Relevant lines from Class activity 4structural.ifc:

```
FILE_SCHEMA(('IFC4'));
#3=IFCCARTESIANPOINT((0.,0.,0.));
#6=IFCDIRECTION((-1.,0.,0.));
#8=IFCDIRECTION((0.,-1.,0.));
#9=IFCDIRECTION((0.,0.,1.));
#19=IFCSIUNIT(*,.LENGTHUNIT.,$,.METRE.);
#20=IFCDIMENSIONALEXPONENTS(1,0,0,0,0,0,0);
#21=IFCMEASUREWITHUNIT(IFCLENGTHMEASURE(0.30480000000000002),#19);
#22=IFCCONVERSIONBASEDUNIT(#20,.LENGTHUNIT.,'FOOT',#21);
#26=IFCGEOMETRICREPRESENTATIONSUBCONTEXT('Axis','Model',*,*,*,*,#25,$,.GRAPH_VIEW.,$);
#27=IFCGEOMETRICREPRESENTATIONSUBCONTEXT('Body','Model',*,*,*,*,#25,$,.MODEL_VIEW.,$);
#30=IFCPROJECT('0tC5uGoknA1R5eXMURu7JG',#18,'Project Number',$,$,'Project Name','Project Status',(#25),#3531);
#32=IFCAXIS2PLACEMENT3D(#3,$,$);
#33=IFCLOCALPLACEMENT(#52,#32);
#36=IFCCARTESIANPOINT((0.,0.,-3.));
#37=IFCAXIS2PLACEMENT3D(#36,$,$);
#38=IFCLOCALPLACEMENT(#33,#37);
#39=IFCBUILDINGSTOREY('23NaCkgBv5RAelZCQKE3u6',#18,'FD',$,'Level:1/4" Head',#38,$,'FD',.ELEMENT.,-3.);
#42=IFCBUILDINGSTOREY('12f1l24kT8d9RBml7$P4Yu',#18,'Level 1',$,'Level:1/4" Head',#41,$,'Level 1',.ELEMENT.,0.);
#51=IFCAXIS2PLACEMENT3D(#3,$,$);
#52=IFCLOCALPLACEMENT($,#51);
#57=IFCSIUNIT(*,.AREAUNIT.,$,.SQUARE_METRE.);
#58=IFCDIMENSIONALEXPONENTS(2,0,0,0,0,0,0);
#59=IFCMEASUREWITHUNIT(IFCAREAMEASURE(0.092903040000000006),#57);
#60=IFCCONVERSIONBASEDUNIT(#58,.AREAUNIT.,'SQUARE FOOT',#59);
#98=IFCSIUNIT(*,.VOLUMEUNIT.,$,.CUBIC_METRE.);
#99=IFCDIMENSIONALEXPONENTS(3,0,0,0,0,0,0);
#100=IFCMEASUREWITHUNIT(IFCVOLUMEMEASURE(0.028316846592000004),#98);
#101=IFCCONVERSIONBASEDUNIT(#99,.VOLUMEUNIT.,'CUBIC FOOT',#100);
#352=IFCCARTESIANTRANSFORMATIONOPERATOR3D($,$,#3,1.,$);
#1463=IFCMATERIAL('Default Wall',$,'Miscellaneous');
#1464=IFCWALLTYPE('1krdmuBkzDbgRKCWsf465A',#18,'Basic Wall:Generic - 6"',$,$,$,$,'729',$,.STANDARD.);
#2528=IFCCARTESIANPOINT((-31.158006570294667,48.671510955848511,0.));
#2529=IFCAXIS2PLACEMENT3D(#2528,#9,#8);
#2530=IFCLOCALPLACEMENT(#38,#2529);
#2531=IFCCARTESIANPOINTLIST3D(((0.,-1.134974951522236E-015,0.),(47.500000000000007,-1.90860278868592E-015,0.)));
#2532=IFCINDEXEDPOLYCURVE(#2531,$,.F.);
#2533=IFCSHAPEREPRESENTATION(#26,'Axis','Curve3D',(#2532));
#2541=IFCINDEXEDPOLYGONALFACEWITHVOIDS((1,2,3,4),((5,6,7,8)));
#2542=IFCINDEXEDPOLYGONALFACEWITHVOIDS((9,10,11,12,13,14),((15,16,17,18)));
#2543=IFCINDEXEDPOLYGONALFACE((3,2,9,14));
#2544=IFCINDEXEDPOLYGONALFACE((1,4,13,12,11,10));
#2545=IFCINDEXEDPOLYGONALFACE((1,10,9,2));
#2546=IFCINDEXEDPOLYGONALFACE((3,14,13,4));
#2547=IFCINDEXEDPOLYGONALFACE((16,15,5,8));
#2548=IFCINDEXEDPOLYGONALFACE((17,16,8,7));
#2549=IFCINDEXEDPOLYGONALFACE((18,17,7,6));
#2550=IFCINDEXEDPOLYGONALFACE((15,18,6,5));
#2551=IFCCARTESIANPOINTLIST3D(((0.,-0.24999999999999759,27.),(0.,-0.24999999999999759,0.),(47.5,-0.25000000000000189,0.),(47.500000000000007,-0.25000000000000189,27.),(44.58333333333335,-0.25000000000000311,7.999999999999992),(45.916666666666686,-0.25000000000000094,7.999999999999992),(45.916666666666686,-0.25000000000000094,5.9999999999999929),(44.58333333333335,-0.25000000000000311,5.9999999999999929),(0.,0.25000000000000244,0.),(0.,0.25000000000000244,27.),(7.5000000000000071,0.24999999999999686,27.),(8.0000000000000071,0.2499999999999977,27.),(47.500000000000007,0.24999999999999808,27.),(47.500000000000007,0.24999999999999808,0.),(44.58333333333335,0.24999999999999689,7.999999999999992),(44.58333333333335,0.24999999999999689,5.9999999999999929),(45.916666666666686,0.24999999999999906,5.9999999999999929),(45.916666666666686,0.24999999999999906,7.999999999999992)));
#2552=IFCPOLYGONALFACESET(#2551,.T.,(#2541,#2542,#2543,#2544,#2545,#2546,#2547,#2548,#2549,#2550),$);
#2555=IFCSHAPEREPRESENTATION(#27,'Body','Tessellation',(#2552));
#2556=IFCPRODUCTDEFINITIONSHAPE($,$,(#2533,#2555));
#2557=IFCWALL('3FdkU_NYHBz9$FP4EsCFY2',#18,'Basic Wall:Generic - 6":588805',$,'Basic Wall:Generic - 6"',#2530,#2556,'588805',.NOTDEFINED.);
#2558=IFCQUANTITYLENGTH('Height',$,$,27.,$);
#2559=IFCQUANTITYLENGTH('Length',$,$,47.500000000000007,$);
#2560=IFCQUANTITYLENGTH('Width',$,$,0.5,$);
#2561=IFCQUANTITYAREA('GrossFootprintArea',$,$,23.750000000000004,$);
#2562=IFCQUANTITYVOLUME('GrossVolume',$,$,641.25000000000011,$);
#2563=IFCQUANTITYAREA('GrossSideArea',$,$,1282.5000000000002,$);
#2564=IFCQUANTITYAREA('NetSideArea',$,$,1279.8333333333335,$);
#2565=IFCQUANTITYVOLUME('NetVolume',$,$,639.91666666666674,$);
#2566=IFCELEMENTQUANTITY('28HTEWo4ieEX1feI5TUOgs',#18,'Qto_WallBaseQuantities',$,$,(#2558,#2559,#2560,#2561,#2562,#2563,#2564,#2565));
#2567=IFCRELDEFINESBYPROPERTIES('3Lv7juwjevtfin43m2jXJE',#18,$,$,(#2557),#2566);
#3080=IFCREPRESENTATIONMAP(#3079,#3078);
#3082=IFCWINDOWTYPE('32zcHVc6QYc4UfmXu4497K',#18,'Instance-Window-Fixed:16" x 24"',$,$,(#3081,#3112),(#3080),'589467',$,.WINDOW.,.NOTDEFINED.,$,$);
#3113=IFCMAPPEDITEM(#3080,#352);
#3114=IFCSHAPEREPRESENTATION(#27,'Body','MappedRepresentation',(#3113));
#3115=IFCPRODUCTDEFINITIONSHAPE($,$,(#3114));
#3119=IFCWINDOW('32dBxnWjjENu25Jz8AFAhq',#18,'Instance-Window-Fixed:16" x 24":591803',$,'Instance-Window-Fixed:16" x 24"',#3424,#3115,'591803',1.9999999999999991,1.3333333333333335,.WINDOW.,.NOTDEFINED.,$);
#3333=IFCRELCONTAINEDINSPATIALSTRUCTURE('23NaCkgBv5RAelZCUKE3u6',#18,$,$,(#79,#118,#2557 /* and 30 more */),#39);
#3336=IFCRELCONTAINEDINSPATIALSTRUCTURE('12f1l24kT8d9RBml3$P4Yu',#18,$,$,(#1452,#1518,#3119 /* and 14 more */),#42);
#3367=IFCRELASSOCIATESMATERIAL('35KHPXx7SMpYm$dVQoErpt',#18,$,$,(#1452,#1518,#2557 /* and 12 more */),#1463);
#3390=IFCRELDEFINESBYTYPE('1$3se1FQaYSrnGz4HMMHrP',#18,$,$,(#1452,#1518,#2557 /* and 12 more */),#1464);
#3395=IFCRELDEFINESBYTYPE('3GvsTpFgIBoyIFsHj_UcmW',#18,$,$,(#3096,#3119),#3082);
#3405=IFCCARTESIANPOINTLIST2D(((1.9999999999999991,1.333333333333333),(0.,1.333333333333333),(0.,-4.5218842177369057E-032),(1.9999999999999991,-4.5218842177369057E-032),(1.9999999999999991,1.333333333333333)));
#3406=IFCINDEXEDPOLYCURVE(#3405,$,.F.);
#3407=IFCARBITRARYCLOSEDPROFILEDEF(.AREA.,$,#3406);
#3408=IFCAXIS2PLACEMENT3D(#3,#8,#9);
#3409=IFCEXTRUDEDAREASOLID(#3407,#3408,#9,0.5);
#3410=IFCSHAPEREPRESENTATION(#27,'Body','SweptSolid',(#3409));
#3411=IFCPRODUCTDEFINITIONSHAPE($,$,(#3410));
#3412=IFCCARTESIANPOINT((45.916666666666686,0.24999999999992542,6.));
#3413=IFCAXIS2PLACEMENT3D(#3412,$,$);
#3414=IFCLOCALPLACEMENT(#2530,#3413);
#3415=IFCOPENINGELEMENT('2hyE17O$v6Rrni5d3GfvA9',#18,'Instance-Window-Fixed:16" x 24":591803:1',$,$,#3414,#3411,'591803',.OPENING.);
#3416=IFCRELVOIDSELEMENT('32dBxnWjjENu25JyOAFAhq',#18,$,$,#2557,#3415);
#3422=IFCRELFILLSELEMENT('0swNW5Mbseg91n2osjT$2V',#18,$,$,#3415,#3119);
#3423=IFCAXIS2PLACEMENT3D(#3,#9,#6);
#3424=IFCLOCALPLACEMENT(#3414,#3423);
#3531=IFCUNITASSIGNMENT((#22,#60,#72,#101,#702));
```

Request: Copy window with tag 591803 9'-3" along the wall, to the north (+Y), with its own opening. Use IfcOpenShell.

```python
import ifcopenshell
import ifcopenshell.api.feature
import ifcopenshell.api.geometry
import ifcopenshell.api.pset
import ifcopenshell.api.root
import ifcopenshell.geom
import ifcopenshell.util.element
import ifcopenshell.util.placement
import ifcopenshell.util.shape
import ifcopenshell.util.unit

model = ifcopenshell.open("Class activity 4structural.ifc")
unit_scale = ifcopenshell.util.unit.calculate_unit_scale(model)
area_scale = ifcopenshell.util.unit.calculate_unit_scale(model, "AREAUNIT")
volume_scale = ifcopenshell.util.unit.calculate_unit_scale(model, "VOLUMEUNIT")
settings = ifcopenshell.geom.settings()


def volume(element):
    """Net volume in cubic metres, openings subtracted."""
    shape = ifcopenshell.geom.create_shape(settings, element)
    return ifcopenshell.util.shape.get_volume(shape.geometry)


def reuse_history(source, copy):
    """copy_class also copies each property set's owner history, people and application; keep the originals."""
    for rel in copy.IsDefinedBy:
        if rel.is_a("IfcRelDefinesByProperties") and (history := rel.RelatingPropertyDefinition.OwnerHistory):
            rel.RelatingPropertyDefinition.OwnerHistory = source.OwnerHistory
            ifcopenshell.util.element.remove_deep2(model, history)


window = model.by_guid("32dBxnWjjENu25Jz8AFAhq")
opening = window.FillsVoids[0].RelatingOpeningElement
wall = opening.VoidsElements[0].RelatingBuildingElement
before = volume(wall)
shift = ifcopenshell.util.placement.get_local_placement(wall.ObjectPlacement)[:3, 0] * -111 * 0.0254 / unit_scale

# copy_class copies the void relationship, type, container and properties, but no geometry.
new_opening = ifcopenshell.api.root.copy_class(model, product=opening)
new_opening.Representation = ifcopenshell.util.element.copy_deep(
    model, opening.Representation, exclude=["IfcGeometricRepresentationContext", "IfcRepresentationMap"]
)
new_opening.Name = 'Instance-Window-Fixed:16" x 24"'
new_opening.Tag = None
reuse_history(opening, new_opening)
new_window = ifcopenshell.api.root.copy_class(model, product=window)
new_window.Representation = ifcopenshell.util.element.copy_deep(
    model, window.Representation, exclude=["IfcGeometricRepresentationContext", "IfcRepresentationMap"]
)
new_window.Name = 'Instance-Window-Fixed:16" x 24"'
new_window.Tag = None
reuse_history(window, new_window)
ifcopenshell.api.feature.add_filling(model, opening=new_opening, element=new_window)

for old, new in ((opening, new_opening), (window, new_window)):
    matrix = ifcopenshell.util.placement.get_local_placement(old.ObjectPlacement)
    matrix[:3, 3] += shift
    ifcopenshell.api.geometry.edit_object_placement(model, product=new, matrix=matrix, is_si=False)

after = volume(wall)
thickness = 0.1524  # wall thickness in metres

# Update the wall's stored quantities.
qto = model.by_id(ifcopenshell.util.element.get_pset(wall, "Qto_WallBaseQuantities", should_inherit=False)["id"])
ifcopenshell.api.pset.edit_qto(model, qto=qto, properties={
    "NetSideArea": after / thickness / area_scale,
    "NetVolume": after / volume_scale,
})

print(f"wall volume {before:.3f} -> {after:.3f} m3")

model.write("Class activity 4structural_edited.ifc")
```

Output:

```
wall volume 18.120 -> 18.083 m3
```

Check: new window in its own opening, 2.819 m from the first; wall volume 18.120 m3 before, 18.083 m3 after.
